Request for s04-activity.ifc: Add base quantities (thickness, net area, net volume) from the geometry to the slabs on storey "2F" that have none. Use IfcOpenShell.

First a look at what the model holds.

```python
import ifcopenshell
import ifcopenshell.util.element
import ifcopenshell.util.unit

model = ifcopenshell.open("s04-activity.ifc")
print(model.schema)
for unit_type in ("LENGTHUNIT", "AREAUNIT", "VOLUMEUNIT"):
    print(unit_type, ifcopenshell.util.unit.calculate_unit_scale(model, unit_type))
storey = next(s for s in model.by_type("IfcBuildingStorey") if s.Name == "2F")
slabs = [e for e in ifcopenshell.util.element.get_decomposition(storey) if e.is_a("IfcSlab")]
for e in sorted(slabs, key=lambda e: e.id()):
    print(e.id(), e.is_a(), e.Name, list(ifcopenshell.util.element.get_psets(e, qtos_only=True)), sep=" | ")
```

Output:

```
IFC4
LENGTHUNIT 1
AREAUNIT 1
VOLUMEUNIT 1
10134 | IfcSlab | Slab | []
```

```python
import ifcopenshell
import ifcopenshell.api.pset
import ifcopenshell.geom
import ifcopenshell.util.element
import ifcopenshell.util.shape
import ifcopenshell.util.unit

model = ifcopenshell.open("s04-activity.ifc")
unit_scale = ifcopenshell.util.unit.calculate_unit_scale(model)
area_scale = ifcopenshell.util.unit.calculate_unit_scale(model, "AREAUNIT")
volume_scale = ifcopenshell.util.unit.calculate_unit_scale(model, "VOLUMEUNIT")
settings = ifcopenshell.geom.settings()

storey = next(s for s in model.by_type("IfcBuildingStorey") if s.Name == "2F")
slabs = [e for e in ifcopenshell.util.element.get_decomposition(storey) if e.is_a("IfcSlab")]

for e in sorted(slabs, key=lambda e: e.id()):
    if ifcopenshell.util.element.get_psets(e, qtos_only=True, should_inherit=False):
        continue
    # Geometry comes back in metres, in the element's own axes.
    shape = ifcopenshell.geom.create_shape(settings, e)
    values = {
        "Width": ifcopenshell.util.shape.get_z(shape.geometry) / unit_scale,
        "NetArea": ifcopenshell.util.shape.get_footprint_area(shape.geometry) / area_scale,
        "NetVolume": ifcopenshell.util.shape.get_volume(shape.geometry) / volume_scale,
    }
    qto = ifcopenshell.api.pset.add_qto(model, product=e, name="Qto_SlabBaseQuantities")
    ifcopenshell.api.pset.edit_qto(model, qto=qto, properties=values)
    print(e.id(), {k: round(v, 3) for k, v in values.items()})

model.write("s04-activity-out.ifc")
```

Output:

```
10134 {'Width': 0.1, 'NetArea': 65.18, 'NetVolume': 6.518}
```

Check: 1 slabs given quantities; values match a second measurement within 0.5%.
